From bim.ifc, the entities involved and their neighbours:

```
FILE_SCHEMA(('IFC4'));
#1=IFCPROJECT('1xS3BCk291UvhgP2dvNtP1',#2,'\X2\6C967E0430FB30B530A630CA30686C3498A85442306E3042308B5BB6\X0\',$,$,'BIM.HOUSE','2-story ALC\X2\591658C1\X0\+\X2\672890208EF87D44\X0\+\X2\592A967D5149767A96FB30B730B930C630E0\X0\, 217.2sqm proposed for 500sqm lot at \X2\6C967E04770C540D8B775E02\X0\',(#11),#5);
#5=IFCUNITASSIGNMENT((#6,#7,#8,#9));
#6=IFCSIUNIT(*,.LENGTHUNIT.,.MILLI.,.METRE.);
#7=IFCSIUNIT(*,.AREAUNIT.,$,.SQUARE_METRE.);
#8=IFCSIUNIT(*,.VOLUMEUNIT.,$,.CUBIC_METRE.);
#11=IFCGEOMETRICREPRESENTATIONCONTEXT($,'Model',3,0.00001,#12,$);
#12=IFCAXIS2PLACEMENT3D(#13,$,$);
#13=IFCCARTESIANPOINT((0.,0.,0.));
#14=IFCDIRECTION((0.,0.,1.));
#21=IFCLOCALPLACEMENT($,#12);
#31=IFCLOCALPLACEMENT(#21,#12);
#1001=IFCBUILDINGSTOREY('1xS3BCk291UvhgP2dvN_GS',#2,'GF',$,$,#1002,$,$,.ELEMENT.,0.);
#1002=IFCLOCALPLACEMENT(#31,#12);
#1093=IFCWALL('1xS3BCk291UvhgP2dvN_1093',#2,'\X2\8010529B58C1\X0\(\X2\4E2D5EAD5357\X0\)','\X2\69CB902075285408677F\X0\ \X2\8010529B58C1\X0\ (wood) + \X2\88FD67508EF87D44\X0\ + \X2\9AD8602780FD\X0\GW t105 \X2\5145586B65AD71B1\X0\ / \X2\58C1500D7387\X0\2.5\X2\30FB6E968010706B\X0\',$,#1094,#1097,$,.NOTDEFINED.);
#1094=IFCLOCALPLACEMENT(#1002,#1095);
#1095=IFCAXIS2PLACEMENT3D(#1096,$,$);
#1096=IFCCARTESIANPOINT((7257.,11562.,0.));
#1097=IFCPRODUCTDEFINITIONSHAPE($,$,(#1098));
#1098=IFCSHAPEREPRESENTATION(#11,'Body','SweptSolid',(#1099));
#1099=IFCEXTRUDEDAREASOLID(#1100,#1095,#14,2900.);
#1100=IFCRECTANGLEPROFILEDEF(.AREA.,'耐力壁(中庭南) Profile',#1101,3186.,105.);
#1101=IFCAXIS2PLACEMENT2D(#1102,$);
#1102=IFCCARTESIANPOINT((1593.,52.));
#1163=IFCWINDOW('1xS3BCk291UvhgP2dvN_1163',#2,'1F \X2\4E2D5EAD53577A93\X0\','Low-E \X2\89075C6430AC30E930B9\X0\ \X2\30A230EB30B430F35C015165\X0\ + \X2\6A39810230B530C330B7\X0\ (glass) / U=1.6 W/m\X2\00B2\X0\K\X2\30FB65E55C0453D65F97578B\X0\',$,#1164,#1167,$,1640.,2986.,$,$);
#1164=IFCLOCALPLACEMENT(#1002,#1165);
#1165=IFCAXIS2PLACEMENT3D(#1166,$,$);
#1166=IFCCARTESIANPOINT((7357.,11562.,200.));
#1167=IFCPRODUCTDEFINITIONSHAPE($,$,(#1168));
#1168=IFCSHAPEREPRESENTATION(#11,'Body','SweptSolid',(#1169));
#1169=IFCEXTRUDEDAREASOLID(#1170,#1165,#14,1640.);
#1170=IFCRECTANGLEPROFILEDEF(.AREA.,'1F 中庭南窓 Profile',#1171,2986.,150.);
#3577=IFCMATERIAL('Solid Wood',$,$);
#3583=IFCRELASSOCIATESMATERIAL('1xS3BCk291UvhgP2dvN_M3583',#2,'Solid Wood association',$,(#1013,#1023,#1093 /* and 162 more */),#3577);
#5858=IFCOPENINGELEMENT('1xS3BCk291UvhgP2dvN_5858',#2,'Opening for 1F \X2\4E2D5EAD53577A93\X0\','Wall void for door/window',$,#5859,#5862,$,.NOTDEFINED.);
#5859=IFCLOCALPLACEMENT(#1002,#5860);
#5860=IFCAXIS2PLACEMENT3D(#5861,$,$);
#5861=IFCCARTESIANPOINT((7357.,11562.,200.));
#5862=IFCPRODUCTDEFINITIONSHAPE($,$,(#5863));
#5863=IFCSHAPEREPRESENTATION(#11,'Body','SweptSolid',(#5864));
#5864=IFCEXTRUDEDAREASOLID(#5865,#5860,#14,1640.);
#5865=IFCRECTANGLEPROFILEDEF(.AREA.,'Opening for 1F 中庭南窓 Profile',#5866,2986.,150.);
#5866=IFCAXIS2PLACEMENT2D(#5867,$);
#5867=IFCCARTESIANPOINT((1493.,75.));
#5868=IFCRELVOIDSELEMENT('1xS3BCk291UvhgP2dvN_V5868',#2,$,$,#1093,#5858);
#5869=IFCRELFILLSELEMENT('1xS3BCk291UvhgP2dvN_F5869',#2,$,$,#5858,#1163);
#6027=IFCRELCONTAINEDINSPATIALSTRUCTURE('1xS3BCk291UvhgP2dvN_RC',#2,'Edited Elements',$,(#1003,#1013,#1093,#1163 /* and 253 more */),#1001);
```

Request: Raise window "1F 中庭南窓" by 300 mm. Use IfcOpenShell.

```python
import numpy as np
import ifcopenshell
import ifcopenshell.api.geometry
import ifcopenshell.util.placement
import ifcopenshell.util.unit

model = ifcopenshell.open("bim.ifc")
unit_scale = ifcopenshell.util.unit.calculate_unit_scale(model)

window = model.by_guid("1xS3BCk291UvhgP2dvN_1163")
opening = window.FillsVoids[0].RelatingOpeningElement
dz = 300.0

shift = np.array([0.0, 0.0, dz])
# The window is not placed relative to its opening, so move both.
for product in (opening, window):
    matrix = ifcopenshell.util.placement.get_local_placement(product.ObjectPlacement)
    matrix[:3, 3] += shift
    ifcopenshell.api.geometry.edit_object_placement(model, product=product, matrix=matrix, is_si=False)

print(f"moved by {dz * unit_scale:+.3f} m")

model.write("bim-out.ifc")
```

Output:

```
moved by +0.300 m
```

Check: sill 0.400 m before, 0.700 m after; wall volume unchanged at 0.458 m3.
